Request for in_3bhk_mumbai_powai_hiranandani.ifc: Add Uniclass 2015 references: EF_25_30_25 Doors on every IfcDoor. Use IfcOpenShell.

First a look at what the model holds.

```python
import ifcopenshell

model = ifcopenshell.open("in_3bhk_mumbai_powai_hiranandani.ifc")
print(model.schema)
print("classifications:", [c.Name for c in model.by_type("IfcClassification")])
for ifc_class in ("IfcDoor", "IfcRoof", "IfcStair", "IfcWall", "IfcWindow"):
    print(ifc_class, len(model.by_type(ifc_class)))
```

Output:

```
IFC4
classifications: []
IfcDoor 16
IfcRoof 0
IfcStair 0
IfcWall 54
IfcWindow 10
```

```python
import ifcopenshell
import ifcopenshell.api.classification

model = ifcopenshell.open("in_3bhk_mumbai_powai_hiranandani.ifc")

system = ifcopenshell.api.classification.add_classification(model, classification="Uniclass 2015")

codes = {
    "IfcDoor": ("EF_25_30_25", "Doors"),
}
for ifc_class, (code, name) in codes.items():
    products = model.by_type(ifc_class)
    ifcopenshell.api.classification.add_reference(
        model, products=products, classification=system, identification=code, name=name
    )
    print(code, len(products))

model.write("in_3bhk_mumbai_powai_hiranandani_rev.ifc")
```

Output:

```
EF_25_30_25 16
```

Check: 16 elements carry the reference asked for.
